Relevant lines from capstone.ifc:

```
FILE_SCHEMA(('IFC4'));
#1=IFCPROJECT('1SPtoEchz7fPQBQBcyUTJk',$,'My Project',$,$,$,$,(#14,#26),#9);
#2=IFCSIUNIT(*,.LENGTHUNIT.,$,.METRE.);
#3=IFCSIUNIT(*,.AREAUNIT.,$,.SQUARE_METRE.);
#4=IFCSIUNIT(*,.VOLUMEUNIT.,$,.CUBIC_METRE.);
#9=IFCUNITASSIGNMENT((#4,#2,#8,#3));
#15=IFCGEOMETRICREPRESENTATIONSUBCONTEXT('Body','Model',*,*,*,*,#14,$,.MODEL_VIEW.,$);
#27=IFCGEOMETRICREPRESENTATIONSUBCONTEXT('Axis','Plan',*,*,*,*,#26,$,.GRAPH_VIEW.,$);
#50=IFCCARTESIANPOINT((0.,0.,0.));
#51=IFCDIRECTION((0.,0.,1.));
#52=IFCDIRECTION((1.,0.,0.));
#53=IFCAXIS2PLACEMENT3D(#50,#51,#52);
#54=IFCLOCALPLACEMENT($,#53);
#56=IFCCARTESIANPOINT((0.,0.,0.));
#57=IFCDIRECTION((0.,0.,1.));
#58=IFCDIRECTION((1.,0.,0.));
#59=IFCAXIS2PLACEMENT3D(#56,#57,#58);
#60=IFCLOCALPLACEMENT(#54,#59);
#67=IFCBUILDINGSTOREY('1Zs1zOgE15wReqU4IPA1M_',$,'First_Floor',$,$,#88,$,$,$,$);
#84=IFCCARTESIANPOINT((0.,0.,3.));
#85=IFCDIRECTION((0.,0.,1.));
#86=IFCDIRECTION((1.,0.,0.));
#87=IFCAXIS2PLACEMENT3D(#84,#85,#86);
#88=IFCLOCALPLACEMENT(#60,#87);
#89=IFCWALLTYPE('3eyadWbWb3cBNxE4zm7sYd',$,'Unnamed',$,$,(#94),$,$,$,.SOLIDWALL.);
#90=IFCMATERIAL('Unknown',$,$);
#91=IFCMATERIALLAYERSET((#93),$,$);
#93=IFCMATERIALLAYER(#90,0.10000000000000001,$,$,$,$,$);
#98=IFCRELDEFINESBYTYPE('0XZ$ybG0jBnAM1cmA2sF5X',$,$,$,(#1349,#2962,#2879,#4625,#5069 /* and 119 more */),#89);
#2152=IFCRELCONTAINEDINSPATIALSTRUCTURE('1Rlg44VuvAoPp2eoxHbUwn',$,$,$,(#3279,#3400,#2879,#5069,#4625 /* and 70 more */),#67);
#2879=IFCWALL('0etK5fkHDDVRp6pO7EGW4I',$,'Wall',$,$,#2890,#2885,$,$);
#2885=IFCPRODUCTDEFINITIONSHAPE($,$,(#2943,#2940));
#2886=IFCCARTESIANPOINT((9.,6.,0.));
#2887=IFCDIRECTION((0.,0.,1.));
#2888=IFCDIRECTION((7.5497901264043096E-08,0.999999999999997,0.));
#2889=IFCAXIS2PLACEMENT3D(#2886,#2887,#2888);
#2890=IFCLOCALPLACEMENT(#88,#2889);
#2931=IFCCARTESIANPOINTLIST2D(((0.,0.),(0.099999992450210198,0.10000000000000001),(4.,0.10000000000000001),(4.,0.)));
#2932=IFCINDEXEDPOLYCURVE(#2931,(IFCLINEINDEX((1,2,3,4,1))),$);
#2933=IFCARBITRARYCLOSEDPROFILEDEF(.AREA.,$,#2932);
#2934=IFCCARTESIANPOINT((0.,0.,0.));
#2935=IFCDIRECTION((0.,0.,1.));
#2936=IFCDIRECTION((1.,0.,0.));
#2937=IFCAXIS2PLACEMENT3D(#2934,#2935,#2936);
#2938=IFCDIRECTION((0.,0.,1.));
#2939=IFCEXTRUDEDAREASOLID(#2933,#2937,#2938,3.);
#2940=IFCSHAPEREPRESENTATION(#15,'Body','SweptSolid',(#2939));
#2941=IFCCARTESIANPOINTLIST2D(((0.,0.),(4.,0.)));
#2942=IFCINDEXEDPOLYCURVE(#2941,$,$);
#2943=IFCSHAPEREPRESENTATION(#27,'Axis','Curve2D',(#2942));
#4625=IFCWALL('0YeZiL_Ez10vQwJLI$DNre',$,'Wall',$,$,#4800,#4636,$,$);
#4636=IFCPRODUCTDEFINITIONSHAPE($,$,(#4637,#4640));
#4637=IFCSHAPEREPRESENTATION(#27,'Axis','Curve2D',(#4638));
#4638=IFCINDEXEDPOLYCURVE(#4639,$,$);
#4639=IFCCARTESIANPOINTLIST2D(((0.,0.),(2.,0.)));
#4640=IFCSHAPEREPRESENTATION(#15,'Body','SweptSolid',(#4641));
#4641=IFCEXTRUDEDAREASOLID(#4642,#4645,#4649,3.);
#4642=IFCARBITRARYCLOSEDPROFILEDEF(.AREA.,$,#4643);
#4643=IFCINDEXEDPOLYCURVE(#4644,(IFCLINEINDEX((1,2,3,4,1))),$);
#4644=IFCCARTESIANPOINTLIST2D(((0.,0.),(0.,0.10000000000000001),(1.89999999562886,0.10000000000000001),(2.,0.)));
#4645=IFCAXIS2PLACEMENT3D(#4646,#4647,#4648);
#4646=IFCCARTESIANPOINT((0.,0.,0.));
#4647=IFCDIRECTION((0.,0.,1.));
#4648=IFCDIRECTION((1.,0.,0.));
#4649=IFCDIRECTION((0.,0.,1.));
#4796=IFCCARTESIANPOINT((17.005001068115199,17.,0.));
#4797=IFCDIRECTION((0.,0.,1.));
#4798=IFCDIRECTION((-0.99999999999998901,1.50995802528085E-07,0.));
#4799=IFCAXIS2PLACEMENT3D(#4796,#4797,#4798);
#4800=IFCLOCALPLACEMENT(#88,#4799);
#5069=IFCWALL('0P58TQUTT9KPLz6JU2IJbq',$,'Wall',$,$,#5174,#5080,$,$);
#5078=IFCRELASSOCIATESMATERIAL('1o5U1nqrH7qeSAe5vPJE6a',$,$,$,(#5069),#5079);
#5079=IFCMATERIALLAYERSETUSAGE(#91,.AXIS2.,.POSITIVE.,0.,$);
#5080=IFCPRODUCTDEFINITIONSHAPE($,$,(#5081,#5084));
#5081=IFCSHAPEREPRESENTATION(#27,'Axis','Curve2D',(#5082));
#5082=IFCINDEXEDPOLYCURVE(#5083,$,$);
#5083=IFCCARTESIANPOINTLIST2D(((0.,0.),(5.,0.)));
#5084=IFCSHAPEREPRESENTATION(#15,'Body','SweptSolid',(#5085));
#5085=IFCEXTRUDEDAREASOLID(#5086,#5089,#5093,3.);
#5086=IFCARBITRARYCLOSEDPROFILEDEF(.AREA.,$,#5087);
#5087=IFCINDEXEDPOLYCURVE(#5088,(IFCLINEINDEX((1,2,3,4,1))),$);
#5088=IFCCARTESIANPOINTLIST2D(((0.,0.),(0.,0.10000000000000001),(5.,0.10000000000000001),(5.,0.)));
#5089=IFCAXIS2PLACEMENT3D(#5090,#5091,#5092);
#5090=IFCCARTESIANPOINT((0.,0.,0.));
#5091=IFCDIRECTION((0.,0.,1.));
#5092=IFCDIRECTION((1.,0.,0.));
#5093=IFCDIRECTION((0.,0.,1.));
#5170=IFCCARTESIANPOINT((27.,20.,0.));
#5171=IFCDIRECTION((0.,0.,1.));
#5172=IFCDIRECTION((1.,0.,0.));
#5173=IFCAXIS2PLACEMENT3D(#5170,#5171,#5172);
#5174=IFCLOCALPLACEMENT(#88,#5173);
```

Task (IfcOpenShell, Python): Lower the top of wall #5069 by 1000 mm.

```python
import ifcopenshell
import ifcopenshell.geom
import ifcopenshell.util.representation
import ifcopenshell.util.shape
import ifcopenshell.util.unit

model = ifcopenshell.open("capstone.ifc")
unit_scale = ifcopenshell.util.unit.calculate_unit_scale(model)
settings = ifcopenshell.geom.settings()


def volume(element):
    """Net volume in cubic metres, openings subtracted."""
    shape = ifcopenshell.geom.create_shape(settings, element)
    return ifcopenshell.util.shape.get_volume(shape.geometry)


wall = model.by_guid("0P58TQUTT9KPLz6JU2IJbq")
before = volume(wall)

body = ifcopenshell.util.representation.get_representation(wall, "Model", "Body")
solid = body.Items[0]
old_height = solid.Depth
solid.Depth -= 1 / unit_scale
after = volume(wall)

print(f"height {old_height:g} -> {solid.Depth:g}, volume {before:.3f} -> {after:.3f} m3")

model.write("capstone_v2.ifc")
```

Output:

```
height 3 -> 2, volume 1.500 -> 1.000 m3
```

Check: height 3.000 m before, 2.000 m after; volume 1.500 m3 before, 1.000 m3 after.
